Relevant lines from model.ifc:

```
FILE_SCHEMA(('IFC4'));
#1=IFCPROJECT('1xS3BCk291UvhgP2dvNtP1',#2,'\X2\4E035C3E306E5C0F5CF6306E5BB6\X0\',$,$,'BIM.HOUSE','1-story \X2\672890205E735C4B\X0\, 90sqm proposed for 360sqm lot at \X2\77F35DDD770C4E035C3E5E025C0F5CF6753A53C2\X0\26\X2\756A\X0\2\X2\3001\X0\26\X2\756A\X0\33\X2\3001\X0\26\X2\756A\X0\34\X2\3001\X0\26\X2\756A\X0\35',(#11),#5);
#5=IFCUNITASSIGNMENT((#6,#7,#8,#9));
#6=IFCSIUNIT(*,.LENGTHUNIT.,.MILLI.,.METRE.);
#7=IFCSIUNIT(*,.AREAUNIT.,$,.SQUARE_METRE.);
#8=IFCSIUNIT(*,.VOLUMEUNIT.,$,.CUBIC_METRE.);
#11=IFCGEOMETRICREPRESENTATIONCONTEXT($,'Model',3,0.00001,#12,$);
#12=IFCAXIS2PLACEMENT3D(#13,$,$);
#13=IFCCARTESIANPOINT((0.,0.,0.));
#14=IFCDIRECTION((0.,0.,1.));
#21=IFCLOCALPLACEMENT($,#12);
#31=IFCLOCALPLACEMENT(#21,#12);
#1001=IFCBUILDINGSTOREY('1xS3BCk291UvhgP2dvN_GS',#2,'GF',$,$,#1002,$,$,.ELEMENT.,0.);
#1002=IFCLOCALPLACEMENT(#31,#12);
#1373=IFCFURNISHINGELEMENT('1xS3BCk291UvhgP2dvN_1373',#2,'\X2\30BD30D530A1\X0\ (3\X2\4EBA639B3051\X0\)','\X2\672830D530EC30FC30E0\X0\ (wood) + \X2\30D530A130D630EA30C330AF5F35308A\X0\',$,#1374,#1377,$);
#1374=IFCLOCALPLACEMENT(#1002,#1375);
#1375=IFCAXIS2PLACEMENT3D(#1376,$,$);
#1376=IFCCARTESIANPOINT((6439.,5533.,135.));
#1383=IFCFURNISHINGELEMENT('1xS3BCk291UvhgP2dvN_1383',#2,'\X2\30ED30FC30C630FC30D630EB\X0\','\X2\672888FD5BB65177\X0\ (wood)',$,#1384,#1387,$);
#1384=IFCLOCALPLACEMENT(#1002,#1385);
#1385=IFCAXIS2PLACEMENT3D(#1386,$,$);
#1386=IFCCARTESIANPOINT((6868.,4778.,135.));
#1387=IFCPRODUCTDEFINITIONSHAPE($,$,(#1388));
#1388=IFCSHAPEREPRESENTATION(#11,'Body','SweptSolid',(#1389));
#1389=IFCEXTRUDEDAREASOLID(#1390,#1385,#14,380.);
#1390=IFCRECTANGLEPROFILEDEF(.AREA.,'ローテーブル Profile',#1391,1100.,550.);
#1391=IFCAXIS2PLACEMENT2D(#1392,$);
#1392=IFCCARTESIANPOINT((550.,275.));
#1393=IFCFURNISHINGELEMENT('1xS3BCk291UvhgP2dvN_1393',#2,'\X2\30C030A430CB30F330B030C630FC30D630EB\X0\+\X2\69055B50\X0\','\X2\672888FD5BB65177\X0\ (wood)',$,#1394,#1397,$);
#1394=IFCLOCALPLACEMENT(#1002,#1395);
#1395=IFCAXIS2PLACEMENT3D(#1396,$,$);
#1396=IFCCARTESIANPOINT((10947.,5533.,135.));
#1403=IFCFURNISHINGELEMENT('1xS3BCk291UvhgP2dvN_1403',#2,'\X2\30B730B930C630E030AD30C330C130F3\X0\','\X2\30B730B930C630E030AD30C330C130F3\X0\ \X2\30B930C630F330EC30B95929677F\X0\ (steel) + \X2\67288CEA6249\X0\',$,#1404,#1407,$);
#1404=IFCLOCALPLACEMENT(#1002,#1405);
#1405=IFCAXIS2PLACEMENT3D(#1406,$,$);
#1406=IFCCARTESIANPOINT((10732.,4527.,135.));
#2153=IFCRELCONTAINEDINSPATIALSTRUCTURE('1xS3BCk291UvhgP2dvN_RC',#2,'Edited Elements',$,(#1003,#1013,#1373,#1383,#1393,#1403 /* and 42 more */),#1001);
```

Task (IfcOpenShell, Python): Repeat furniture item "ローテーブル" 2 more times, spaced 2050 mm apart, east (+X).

```python
import numpy as np
import ifcopenshell
import ifcopenshell.api.geometry
import ifcopenshell.api.root
import ifcopenshell.util.element
import ifcopenshell.util.placement

model = ifcopenshell.open("model.ifc")


def reuse_history(source, copy):
    """copy_class also copies each property set's owner history, people and application; keep the originals."""
    for rel in copy.IsDefinedBy:
        if rel.is_a("IfcRelDefinesByProperties") and (history := rel.RelatingPropertyDefinition.OwnerHistory):
            rel.RelatingPropertyDefinition.OwnerHistory = source.OwnerHistory
            ifcopenshell.util.element.remove_deep2(model, history)


source = model.by_guid("1xS3BCk291UvhgP2dvN_1383")
base = ifcopenshell.util.placement.get_local_placement(source.ObjectPlacement)
step = np.array([1.0, 0.0, 0.0]) * 2050.0

for i in range(1, 3):
    copy = ifcopenshell.api.root.copy_class(model, product=source)
    copy.Representation = ifcopenshell.util.element.copy_deep(
        model, source.Representation, exclude=["IfcGeometricRepresentationContext", "IfcRepresentationMap"]
    )
    reuse_history(source, copy)
    matrix = base.copy()
    matrix[:3, 3] += i * step
    print("added at", matrix[:3, 3].round(3) + 0.0)
    ifcopenshell.api.geometry.edit_object_placement(model, product=copy, matrix=matrix, is_si=False)

model.write("model_updated.ifc")
```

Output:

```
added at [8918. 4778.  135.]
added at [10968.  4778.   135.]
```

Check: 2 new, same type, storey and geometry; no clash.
